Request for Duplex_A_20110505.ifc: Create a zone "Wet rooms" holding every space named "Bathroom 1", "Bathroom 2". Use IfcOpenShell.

First a look at what the model holds.

```python
import ifcopenshell

model = ifcopenshell.open("Duplex_A_20110505.ifc")
print(model.schema)
seen = {}
for space in model.by_type("IfcSpace"):
    seen[space.LongName] = seen.get(space.LongName, 0) + 1
for name, count in sorted(seen.items(), key=str):
    print(count, "x", name)
print("zones:", [z.Name for z in model.by_type("IfcZone")][:20])
```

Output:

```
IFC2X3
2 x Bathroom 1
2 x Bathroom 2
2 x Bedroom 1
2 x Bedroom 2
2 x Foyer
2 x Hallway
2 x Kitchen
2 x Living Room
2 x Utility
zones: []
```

```python
import ifcopenshell
import ifcopenshell.api.group
import ifcopenshell.api.root

model = ifcopenshell.open("Duplex_A_20110505.ifc")

names = {"Bathroom 1", "Bathroom 2"}
spaces = [s for s in model.by_type("IfcSpace") if s.LongName in names]

zone = ifcopenshell.api.root.create_entity(model, ifc_class="IfcZone", name="Wet rooms")
ifcopenshell.api.group.assign_group(model, products=spaces, group=zone)
print(len(spaces), "spaces in", zone.Name)

model.write("Duplex_A_20110505_rev.ifc")
```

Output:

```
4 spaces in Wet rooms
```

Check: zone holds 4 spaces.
